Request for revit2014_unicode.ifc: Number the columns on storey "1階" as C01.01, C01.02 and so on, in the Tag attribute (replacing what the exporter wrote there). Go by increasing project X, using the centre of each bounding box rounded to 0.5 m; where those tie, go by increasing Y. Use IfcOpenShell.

First a look at what the model holds.

```python
import ifcopenshell
import ifcopenshell.util.element
import ifcopenshell.util.placement

model = ifcopenshell.open("revit2014_unicode.ifc")
print(model.schema)
storey = next(s for s in model.by_type("IfcBuildingStorey") if s.Name == "1階")
columns = [e for e in ifcopenshell.util.element.get_decomposition(storey) if e.is_a("IfcColumn")]
for e in sorted(columns, key=lambda e: e.id()):
    origin = ifcopenshell.util.placement.get_local_placement(e.ObjectPlacement)[:3, 3]
    print(e.id(), e.Tag, e.Name, origin.round(2) + 0.0, sep=" | ")
```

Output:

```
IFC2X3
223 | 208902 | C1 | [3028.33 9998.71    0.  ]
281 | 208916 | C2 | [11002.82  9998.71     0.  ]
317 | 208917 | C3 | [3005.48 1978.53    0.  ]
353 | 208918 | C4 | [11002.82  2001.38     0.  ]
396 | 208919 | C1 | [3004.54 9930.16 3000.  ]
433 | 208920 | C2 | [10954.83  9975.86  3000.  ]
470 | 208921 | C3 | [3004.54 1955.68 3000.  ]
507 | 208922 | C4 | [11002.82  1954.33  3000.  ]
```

```python
import ifcopenshell
import ifcopenshell.geom
import ifcopenshell.util.element
import ifcopenshell.util.shape

model = ifcopenshell.open("revit2014_unicode.ifc")
settings = ifcopenshell.geom.settings()
settings.set("use-world-coords", True)


def centre(element):
    shape = ifcopenshell.geom.create_shape(settings, element)
    return ifcopenshell.util.shape.get_bbox_centroid(shape.geometry)


storey = next(s for s in model.by_type("IfcBuildingStorey") if s.Name == "1階")
columns = [e for e in ifcopenshell.util.element.get_decomposition(storey) if e.is_a("IfcColumn")]

# Insertion points can sit at a corner or the storey origin, so sort by the geometry (in metres).
centres = {e: centre(e) for e in columns}
columns.sort(key=lambda e: (round(centres[e][0] / 0.5), centres[e][1]))

for i, e in enumerate(columns, start=1):
    number = f"C01.{i:02d}"
    e.Tag = number
    print(e.id(), number)

model.write("revit2014_unicode_updated.ifc")
```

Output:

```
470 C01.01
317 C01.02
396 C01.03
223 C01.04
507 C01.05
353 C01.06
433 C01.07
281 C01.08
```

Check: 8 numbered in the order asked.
